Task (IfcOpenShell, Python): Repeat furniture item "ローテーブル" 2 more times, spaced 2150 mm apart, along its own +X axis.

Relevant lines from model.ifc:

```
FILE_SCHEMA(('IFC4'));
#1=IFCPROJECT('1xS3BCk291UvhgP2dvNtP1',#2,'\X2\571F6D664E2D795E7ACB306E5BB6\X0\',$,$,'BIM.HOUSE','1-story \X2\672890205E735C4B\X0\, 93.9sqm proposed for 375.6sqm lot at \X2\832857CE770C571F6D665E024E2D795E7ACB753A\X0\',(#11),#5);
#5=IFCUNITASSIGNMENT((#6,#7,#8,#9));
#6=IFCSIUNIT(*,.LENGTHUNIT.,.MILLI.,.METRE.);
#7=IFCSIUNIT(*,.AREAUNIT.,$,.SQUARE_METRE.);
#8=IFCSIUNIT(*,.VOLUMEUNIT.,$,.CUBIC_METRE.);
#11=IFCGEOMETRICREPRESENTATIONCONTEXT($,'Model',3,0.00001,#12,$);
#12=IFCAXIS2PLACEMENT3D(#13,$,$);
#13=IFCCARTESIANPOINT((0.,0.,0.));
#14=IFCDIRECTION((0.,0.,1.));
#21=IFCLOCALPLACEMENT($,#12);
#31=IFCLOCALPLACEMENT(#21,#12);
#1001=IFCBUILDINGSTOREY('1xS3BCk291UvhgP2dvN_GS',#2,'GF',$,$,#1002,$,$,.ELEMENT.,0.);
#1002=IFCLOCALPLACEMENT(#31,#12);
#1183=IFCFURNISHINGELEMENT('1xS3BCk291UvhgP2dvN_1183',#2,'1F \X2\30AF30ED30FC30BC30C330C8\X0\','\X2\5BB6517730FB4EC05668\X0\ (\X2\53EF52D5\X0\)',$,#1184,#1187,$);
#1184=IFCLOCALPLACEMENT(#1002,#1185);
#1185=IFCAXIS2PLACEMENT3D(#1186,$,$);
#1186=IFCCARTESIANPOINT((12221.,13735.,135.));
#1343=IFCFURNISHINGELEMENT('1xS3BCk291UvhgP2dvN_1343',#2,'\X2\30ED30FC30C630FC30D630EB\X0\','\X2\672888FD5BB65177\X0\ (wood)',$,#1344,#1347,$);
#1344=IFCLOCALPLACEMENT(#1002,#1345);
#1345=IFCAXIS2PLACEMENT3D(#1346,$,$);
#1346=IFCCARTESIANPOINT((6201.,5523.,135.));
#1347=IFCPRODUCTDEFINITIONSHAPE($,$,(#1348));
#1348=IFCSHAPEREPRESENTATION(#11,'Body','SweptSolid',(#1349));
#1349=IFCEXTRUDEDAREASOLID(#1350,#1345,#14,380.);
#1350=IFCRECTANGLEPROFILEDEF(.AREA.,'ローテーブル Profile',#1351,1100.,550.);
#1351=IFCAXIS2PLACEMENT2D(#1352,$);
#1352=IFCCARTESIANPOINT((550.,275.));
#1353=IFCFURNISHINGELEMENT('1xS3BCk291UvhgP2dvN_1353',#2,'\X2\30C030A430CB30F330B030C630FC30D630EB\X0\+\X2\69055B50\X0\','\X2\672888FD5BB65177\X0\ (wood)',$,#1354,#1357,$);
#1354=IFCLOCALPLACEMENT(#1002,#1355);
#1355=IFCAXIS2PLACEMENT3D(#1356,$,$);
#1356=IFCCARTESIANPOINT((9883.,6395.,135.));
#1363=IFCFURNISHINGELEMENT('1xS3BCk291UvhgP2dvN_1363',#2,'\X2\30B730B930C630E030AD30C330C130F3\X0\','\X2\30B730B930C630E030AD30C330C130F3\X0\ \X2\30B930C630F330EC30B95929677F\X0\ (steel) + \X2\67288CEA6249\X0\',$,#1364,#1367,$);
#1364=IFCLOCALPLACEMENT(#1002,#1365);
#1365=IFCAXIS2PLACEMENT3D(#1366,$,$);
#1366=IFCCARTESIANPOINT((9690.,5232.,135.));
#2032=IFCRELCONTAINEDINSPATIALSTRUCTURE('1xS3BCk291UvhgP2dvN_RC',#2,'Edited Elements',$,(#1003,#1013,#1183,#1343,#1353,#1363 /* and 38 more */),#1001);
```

```python
import ifcopenshell
import ifcopenshell.api.geometry
import ifcopenshell.api.root
import ifcopenshell.util.element
import ifcopenshell.util.placement
import ifcopenshell.util.unit

model = ifcopenshell.open("model.ifc")
unit_scale = ifcopenshell.util.unit.calculate_unit_scale(model)


def reuse_history(source, copy):
    """copy_class also copies each property set's owner history, people and application; keep the originals."""
    for rel in copy.IsDefinedBy:
        if rel.is_a("IfcRelDefinesByProperties") and (history := rel.RelatingPropertyDefinition.OwnerHistory):
            rel.RelatingPropertyDefinition.OwnerHistory = source.OwnerHistory
            ifcopenshell.util.element.remove_deep2(model, history)


source = model.by_id(1343)
base = ifcopenshell.util.placement.get_local_placement(source.ObjectPlacement)
step = base[:3, 0] * 2.15 / unit_scale

for i in range(1, 3):
    copy = ifcopenshell.api.root.copy_class(model, product=source)
    copy.Representation = ifcopenshell.util.element.copy_deep(
        model, source.Representation, exclude=["IfcGeometricRepresentationContext", "IfcRepresentationMap"]
    )
    reuse_history(source, copy)
    matrix = base.copy()
    matrix[:3, 3] += i * step
    print("added at", matrix[:3, 3].round(3) + 0.0)
    ifcopenshell.api.geometry.edit_object_placement(model, product=copy, matrix=matrix, is_si=False)

model.write("model_rev.ifc")
```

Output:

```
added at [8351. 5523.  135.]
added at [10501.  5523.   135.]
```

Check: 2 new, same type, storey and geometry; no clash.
